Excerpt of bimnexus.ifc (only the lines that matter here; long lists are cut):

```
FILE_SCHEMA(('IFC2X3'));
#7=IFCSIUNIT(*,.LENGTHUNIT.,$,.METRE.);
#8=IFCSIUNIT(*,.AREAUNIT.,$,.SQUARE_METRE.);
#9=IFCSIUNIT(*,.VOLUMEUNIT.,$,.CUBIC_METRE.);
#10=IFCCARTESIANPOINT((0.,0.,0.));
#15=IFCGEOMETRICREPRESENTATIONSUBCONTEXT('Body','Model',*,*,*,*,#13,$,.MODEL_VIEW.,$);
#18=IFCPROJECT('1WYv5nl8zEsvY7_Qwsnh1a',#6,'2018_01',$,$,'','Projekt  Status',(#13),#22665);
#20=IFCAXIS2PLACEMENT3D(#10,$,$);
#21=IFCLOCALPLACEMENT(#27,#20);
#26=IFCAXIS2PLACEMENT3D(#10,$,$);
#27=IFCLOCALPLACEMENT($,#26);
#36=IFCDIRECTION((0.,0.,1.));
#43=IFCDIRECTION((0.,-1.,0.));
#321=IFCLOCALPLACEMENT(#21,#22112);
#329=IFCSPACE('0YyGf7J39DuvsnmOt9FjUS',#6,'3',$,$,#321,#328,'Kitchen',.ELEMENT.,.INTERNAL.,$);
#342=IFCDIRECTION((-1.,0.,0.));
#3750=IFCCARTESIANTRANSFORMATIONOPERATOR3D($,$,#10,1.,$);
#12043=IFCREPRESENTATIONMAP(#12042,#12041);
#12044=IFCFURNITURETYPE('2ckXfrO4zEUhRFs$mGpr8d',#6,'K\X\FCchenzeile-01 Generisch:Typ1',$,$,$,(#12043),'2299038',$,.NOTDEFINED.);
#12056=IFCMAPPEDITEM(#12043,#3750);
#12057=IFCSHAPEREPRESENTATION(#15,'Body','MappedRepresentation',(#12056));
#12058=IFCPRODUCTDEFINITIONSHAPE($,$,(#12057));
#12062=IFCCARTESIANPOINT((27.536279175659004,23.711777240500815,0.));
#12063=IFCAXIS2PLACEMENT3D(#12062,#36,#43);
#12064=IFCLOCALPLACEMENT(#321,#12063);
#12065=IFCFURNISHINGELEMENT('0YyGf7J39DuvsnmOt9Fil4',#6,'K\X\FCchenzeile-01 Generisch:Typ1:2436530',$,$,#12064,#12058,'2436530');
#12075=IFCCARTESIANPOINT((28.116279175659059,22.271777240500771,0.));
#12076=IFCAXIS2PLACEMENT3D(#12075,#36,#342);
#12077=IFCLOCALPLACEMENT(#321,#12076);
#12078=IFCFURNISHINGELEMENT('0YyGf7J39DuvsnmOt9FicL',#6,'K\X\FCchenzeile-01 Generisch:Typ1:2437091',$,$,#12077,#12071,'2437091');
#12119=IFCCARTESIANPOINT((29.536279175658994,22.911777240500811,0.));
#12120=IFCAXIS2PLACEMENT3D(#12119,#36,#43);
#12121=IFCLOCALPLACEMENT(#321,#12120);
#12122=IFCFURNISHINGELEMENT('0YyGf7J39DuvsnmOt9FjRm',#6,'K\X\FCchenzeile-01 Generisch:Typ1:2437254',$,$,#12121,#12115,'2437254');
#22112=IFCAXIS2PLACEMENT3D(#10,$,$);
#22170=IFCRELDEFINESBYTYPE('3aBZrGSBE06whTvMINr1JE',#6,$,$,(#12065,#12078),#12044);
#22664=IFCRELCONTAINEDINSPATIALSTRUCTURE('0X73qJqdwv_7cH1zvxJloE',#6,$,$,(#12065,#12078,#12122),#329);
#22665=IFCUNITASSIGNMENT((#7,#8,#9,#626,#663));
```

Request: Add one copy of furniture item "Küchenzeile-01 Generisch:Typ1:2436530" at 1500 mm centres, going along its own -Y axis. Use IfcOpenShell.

```python
import ifcopenshell
import ifcopenshell.api.geometry
import ifcopenshell.api.root
import ifcopenshell.util.element
import ifcopenshell.util.placement

model = ifcopenshell.open("bimnexus.ifc")


def reuse_history(source, copy):
    """copy_class also copies each property set's owner history, people and application; keep the originals."""
    for rel in copy.IsDefinedBy:
        if rel.is_a("IfcRelDefinesByProperties") and (history := rel.RelatingPropertyDefinition.OwnerHistory):
            rel.RelatingPropertyDefinition.OwnerHistory = source.OwnerHistory
            ifcopenshell.util.element.remove_deep2(model, history)


source = model.by_guid("0YyGf7J39DuvsnmOt9Fil4")
base = ifcopenshell.util.placement.get_local_placement(source.ObjectPlacement)
step = -base[:3, 1] * 1.5

for i in range(1, 2):
    copy = ifcopenshell.api.root.copy_class(model, product=source)
    copy.Representation = ifcopenshell.util.element.copy_deep(
        model, source.Representation, exclude=["IfcGeometricRepresentationContext", "IfcRepresentationMap"]
    )
    copy.Name = "Küchenzeile-01 Generisch:Typ1"
    copy.Tag = None
    reuse_history(source, copy)
    matrix = base.copy()
    matrix[:3, 3] += i * step
    print("added at", matrix[:3, 3].round(3) + 0.0)
    ifcopenshell.api.geometry.edit_object_placement(model, product=copy, matrix=matrix, is_si=False)

model.write("bimnexus_rev.ifc")
```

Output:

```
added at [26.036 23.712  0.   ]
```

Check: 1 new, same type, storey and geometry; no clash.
